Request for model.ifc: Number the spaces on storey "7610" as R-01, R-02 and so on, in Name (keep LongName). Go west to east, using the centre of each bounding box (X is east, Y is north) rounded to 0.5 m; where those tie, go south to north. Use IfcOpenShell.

First a look at what the model holds.

```python
import ifcopenshell
import ifcopenshell.util.element
import ifcopenshell.util.placement

model = ifcopenshell.open("model.ifc")
print(model.schema)
storey = next(s for s in model.by_type("IfcBuildingStorey") if s.Name == "7610")
spaces = [e for e in ifcopenshell.util.element.get_decomposition(storey) if e.is_a("IfcSpace")]
for e in sorted(spaces, key=lambda e: e.id()):
    origin = ifcopenshell.util.placement.get_local_placement(e.ObjectPlacement)[:3, 3]
    print(e.id(), e.Name, e.LongName, origin.round(2) + 0.0, sep=" | ")
```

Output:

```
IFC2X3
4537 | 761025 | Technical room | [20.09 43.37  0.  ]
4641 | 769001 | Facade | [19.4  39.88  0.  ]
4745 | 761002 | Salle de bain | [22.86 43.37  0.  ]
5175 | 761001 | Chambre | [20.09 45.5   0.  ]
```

```python
import ifcopenshell
import ifcopenshell.geom
import ifcopenshell.util.element
import ifcopenshell.util.shape

model = ifcopenshell.open("model.ifc")
settings = ifcopenshell.geom.settings()
settings.set("use-world-coords", True)


def centre(element):
    shape = ifcopenshell.geom.create_shape(settings, element)
    return ifcopenshell.util.shape.get_bbox_centroid(shape.geometry)


storey = next(s for s in model.by_type("IfcBuildingStorey") if s.Name == "7610")
spaces = [e for e in ifcopenshell.util.element.get_decomposition(storey) if e.is_a("IfcSpace")]

# Insertion points can sit at a corner or the storey origin, so sort by the geometry (in metres).
centres = {e: centre(e) for e in spaces}
spaces.sort(key=lambda e: (round(centres[e][0] / 0.5), centres[e][1]))

for i, e in enumerate(spaces, start=1):
    number = f"R-{i:02d}"
    e.Name = number
    print(e.id(), number)

model.write("model_v2.ifc")
```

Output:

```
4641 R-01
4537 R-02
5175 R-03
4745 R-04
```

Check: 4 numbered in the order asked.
